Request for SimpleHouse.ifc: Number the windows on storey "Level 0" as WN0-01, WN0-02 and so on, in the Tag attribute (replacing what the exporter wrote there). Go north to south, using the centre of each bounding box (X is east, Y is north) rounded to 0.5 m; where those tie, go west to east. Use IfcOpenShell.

First a look at what the model holds.

```python
import ifcopenshell
import ifcopenshell.util.element
import ifcopenshell.util.placement

model = ifcopenshell.open("SimpleHouse.ifc")
print(model.schema)
storey = next(s for s in model.by_type("IfcBuildingStorey") if s.Name == "Level 0")
windows = [e for e in ifcopenshell.util.element.get_decomposition(storey) if e.is_a("IfcWindow")]
for e in sorted(windows, key=lambda e: e.id()):
    origin = ifcopenshell.util.placement.get_local_placement(e.ObjectPlacement)[:3, 3]
    print(e.id(), e.Tag, e.Name, origin.round(2) + 0.0, sep=" | ")
```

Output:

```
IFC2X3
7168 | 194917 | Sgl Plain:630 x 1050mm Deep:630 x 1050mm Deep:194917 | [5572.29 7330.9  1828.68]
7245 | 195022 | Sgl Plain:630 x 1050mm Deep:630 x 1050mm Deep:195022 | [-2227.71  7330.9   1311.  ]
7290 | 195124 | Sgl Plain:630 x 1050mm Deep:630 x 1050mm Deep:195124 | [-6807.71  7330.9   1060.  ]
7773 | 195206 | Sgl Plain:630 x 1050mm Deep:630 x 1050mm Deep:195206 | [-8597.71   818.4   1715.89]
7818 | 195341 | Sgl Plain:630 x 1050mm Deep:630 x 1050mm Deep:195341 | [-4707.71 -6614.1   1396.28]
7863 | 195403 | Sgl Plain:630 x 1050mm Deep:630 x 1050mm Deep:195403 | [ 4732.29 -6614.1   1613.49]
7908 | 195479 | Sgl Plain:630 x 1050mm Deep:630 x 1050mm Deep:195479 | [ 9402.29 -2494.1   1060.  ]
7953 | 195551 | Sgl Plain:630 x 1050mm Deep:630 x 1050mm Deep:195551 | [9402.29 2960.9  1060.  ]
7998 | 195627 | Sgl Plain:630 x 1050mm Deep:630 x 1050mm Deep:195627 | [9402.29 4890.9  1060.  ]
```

```python
import ifcopenshell
import ifcopenshell.geom
import ifcopenshell.util.element
import ifcopenshell.util.shape

model = ifcopenshell.open("SimpleHouse.ifc")
settings = ifcopenshell.geom.settings()
settings.set("use-world-coords", True)


def centre(element):
    shape = ifcopenshell.geom.create_shape(settings, element)
    return ifcopenshell.util.shape.get_bbox_centroid(shape.geometry)


storey = next(s for s in model.by_type("IfcBuildingStorey") if s.Name == "Level 0")
windows = [e for e in ifcopenshell.util.element.get_decomposition(storey) if e.is_a("IfcWindow")]

# Insertion points can sit at a corner or the storey origin, so sort by the geometry (in metres).
centres = {e: centre(e) for e in windows}
windows.sort(key=lambda e: (-round(centres[e][1] / 0.5), centres[e][0]))

for i, e in enumerate(windows, start=1):
    number = f"WN0-{i:02d}"
    e.Tag = number
    print(e.id(), number)

model.write("SimpleHouse_edited.ifc")
```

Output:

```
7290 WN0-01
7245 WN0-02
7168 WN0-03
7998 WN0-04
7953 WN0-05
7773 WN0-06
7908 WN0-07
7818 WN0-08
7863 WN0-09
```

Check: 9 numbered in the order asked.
